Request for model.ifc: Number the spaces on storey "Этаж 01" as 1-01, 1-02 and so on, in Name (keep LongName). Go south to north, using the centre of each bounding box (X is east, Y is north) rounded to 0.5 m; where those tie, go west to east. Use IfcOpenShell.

First a look at what the model holds.

```python
import ifcopenshell
import ifcopenshell.util.element
import ifcopenshell.util.placement

model = ifcopenshell.open("model.ifc")
print(model.schema)
storey = next(s for s in model.by_type("IfcBuildingStorey") if s.Name == "Этаж 01")
spaces = [e for e in ifcopenshell.util.element.get_decomposition(storey) if e.is_a("IfcSpace")]
for e in sorted(spaces, key=lambda e: e.id()):
    origin = ifcopenshell.util.placement.get_local_placement(e.ObjectPlacement)[:3, 3]
    print(e.id(), e.Name, e.LongName, origin.round(2) + 0.0, sep=" | ")
```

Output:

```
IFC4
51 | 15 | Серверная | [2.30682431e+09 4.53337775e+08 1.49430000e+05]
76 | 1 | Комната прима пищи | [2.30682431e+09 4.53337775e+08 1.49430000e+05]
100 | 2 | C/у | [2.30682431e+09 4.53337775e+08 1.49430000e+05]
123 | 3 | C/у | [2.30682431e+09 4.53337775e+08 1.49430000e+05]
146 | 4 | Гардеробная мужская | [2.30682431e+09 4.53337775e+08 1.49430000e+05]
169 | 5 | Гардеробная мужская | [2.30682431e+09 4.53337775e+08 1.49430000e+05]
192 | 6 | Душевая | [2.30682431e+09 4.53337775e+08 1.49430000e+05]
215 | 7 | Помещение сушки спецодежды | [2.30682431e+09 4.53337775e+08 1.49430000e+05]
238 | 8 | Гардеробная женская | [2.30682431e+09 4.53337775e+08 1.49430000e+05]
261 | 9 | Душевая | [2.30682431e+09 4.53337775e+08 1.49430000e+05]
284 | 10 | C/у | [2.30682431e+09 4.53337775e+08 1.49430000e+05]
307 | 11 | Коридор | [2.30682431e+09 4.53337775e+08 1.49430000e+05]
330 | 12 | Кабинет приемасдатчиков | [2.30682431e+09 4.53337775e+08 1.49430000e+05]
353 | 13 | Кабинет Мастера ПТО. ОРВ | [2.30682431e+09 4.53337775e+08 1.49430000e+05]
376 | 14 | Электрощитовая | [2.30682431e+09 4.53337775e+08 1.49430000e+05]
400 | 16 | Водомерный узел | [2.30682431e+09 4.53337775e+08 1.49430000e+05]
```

```python
import ifcopenshell
import ifcopenshell.geom
import ifcopenshell.util.element
import ifcopenshell.util.shape

model = ifcopenshell.open("model.ifc")
settings = ifcopenshell.geom.settings()
settings.set("use-world-coords", True)


def centre(element):
    shape = ifcopenshell.geom.create_shape(settings, element)
    return ifcopenshell.util.shape.get_bbox_centroid(shape.geometry)


storey = next(s for s in model.by_type("IfcBuildingStorey") if s.Name == "Этаж 01")
spaces = [e for e in ifcopenshell.util.element.get_decomposition(storey) if e.is_a("IfcSpace")]

# Insertion points can sit at a corner or the storey origin, so sort by the geometry (in metres).
centres = {e: centre(e) for e in spaces}
spaces.sort(key=lambda e: (round(centres[e][1] / 0.5), centres[e][0]))

for i, e in enumerate(spaces, start=1):
    number = f"1-{i:02d}"
    e.Name = number
    print(e.id(), number)

model.write("model_v2.ifc")
```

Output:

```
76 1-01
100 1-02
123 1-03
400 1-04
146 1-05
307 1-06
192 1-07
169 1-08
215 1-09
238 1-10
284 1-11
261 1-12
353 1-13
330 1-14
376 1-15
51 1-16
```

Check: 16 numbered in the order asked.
